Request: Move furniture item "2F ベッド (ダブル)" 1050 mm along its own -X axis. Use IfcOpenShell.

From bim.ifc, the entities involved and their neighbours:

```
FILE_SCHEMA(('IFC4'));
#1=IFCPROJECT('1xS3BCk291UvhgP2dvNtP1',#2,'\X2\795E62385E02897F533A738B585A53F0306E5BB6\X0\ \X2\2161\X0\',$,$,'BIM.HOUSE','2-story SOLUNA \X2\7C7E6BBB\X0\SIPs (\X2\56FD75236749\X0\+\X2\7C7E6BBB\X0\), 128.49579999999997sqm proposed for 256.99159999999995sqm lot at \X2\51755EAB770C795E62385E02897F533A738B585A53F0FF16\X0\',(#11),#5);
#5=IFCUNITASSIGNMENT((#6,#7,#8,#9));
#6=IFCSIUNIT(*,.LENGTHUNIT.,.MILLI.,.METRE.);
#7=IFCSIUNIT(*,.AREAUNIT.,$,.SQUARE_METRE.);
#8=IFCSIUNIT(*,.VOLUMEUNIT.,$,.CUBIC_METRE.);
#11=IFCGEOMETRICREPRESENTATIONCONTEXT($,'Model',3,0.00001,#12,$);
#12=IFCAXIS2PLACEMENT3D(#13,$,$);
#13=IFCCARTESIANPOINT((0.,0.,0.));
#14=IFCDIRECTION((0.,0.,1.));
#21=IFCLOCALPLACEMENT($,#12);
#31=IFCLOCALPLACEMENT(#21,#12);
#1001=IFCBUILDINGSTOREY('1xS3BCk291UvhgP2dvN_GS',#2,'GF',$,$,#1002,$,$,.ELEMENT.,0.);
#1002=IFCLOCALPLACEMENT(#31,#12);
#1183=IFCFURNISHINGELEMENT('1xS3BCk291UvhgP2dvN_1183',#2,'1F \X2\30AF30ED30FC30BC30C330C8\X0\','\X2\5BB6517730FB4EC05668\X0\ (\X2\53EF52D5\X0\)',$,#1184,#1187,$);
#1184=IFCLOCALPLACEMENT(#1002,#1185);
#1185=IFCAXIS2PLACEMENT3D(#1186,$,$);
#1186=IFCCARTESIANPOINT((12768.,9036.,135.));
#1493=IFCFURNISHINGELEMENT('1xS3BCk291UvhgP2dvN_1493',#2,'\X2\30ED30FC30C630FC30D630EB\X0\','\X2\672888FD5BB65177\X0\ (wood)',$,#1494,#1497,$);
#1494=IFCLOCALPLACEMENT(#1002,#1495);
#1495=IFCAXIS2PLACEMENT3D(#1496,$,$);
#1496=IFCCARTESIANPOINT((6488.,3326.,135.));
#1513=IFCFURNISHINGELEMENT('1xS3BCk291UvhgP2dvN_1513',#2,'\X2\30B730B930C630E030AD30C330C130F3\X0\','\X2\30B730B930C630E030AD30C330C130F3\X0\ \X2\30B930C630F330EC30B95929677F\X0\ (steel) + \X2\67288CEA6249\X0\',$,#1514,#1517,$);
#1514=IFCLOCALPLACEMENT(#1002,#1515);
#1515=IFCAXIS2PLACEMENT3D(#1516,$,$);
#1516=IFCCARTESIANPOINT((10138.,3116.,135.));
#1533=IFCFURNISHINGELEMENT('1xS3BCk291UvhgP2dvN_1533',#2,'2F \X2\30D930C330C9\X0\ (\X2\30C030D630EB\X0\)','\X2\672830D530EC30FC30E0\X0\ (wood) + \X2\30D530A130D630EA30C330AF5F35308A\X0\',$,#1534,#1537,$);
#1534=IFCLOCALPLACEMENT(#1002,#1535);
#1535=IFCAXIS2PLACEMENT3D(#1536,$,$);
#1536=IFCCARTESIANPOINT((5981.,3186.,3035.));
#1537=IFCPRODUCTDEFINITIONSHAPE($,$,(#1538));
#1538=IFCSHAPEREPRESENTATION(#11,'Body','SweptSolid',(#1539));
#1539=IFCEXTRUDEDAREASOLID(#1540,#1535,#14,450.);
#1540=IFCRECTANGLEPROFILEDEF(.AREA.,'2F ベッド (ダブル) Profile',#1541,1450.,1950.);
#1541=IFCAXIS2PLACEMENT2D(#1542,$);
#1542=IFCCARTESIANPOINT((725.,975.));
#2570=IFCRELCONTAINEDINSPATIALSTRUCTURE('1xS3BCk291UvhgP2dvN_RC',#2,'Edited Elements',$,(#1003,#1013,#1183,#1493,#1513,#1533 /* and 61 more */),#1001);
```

```python
import ifcopenshell
import ifcopenshell.api.geometry
import ifcopenshell.util.placement

model = ifcopenshell.open("bim.ifc")

item = model.by_guid("1xS3BCk291UvhgP2dvN_1533")
matrix = ifcopenshell.util.placement.get_local_placement(item.ObjectPlacement)
matrix[:3, 3] -= matrix[:3, 0] * 1050.0
ifcopenshell.api.geometry.edit_object_placement(model, product=item, matrix=matrix, is_si=False)

print(ifcopenshell.util.placement.get_local_placement(item.ObjectPlacement).round(3) + 0.0)

model.write("bim_updated.ifc")
```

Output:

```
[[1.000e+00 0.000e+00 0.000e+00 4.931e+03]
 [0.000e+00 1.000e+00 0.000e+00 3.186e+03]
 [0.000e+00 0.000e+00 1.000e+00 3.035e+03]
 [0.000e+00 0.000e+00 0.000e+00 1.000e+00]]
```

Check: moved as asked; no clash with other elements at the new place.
